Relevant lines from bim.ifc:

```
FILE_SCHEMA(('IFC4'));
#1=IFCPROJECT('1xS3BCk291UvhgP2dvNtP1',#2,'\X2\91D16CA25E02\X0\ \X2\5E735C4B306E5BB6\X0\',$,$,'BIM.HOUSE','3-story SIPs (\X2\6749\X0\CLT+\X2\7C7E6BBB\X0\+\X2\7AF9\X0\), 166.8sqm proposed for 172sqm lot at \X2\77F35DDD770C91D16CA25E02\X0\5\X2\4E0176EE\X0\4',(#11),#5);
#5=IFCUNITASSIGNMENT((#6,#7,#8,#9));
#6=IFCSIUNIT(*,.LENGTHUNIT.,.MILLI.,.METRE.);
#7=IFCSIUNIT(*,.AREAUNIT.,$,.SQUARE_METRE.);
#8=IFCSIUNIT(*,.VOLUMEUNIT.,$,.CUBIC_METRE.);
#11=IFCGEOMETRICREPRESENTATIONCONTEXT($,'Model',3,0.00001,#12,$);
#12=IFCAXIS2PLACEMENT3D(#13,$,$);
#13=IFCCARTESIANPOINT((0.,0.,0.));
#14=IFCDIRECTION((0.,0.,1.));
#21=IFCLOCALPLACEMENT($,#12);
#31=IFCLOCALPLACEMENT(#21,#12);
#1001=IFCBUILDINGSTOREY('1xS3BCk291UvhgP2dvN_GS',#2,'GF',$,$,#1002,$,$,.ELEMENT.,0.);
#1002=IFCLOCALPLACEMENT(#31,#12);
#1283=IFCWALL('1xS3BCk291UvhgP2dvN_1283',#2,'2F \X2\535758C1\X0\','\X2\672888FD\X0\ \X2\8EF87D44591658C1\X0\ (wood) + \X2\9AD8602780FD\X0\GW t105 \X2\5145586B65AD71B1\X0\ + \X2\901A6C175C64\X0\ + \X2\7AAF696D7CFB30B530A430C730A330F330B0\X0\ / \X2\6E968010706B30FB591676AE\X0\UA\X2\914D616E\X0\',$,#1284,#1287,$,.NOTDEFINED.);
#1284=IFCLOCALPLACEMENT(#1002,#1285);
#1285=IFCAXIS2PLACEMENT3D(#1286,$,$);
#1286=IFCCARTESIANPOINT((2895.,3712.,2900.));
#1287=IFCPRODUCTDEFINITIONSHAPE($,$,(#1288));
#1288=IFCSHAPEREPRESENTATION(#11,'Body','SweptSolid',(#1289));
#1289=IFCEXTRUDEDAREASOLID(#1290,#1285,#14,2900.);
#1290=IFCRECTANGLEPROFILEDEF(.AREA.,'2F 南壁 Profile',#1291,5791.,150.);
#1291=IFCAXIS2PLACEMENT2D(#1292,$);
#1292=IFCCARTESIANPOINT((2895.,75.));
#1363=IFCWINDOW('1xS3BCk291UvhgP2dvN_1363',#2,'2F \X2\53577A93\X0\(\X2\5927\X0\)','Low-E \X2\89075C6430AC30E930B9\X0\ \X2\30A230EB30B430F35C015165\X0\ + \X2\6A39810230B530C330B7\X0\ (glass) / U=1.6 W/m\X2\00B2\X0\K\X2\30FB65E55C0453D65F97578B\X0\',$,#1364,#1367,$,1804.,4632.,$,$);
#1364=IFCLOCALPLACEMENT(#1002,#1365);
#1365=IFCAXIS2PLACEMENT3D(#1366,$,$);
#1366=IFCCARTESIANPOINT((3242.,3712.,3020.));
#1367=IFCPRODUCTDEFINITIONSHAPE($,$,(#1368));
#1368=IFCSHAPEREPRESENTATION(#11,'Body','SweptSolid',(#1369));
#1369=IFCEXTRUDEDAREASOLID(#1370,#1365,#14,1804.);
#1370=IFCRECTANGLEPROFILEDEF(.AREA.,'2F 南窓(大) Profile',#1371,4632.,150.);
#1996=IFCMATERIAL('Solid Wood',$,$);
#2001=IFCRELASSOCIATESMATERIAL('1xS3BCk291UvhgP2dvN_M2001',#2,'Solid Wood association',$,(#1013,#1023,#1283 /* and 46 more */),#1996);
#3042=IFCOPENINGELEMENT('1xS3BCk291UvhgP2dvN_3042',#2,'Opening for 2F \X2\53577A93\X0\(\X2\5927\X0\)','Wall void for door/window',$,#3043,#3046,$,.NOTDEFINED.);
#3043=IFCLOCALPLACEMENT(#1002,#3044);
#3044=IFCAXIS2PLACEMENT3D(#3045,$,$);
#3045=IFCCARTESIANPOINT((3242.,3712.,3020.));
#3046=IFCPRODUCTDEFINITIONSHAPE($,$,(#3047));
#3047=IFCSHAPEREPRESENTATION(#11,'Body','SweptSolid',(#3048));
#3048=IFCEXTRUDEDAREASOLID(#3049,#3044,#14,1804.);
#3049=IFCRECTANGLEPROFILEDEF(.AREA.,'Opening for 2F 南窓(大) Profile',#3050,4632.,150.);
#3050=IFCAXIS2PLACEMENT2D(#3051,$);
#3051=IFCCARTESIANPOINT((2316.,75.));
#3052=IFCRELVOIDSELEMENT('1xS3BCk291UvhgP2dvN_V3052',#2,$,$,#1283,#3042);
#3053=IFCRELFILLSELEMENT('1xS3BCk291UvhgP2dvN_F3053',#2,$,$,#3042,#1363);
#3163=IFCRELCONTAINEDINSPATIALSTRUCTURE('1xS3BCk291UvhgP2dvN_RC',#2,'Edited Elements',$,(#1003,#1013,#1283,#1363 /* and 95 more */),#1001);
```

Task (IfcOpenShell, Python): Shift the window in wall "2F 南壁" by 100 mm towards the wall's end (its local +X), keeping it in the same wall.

```python
import ifcopenshell
import ifcopenshell.api.geometry
import ifcopenshell.util.placement

model = ifcopenshell.open("bim.ifc")

window = model.by_guid("1xS3BCk291UvhgP2dvN_1363")
opening = window.FillsVoids[0].RelatingOpeningElement
wall = opening.VoidsElements[0].RelatingBuildingElement

wall_matrix = ifcopenshell.util.placement.get_local_placement(wall.ObjectPlacement)
shift = wall_matrix[:3, 0] * 100.0
before = ifcopenshell.util.placement.get_local_placement(window.ObjectPlacement)[:3, 3].copy()

# The window is not placed relative to its opening, so move both.
for product in (opening, window):
    matrix = ifcopenshell.util.placement.get_local_placement(product.ObjectPlacement)
    matrix[:3, 3] += shift
    ifcopenshell.api.geometry.edit_object_placement(model, product=product, matrix=matrix, is_si=False)

after = ifcopenshell.util.placement.get_local_placement(window.ObjectPlacement)[:3, 3]
print("window moved by", (after - before).round(3) + 0.0)

model.write("bim_edited.ifc")
```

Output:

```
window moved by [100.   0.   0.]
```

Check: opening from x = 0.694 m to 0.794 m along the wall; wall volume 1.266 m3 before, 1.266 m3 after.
